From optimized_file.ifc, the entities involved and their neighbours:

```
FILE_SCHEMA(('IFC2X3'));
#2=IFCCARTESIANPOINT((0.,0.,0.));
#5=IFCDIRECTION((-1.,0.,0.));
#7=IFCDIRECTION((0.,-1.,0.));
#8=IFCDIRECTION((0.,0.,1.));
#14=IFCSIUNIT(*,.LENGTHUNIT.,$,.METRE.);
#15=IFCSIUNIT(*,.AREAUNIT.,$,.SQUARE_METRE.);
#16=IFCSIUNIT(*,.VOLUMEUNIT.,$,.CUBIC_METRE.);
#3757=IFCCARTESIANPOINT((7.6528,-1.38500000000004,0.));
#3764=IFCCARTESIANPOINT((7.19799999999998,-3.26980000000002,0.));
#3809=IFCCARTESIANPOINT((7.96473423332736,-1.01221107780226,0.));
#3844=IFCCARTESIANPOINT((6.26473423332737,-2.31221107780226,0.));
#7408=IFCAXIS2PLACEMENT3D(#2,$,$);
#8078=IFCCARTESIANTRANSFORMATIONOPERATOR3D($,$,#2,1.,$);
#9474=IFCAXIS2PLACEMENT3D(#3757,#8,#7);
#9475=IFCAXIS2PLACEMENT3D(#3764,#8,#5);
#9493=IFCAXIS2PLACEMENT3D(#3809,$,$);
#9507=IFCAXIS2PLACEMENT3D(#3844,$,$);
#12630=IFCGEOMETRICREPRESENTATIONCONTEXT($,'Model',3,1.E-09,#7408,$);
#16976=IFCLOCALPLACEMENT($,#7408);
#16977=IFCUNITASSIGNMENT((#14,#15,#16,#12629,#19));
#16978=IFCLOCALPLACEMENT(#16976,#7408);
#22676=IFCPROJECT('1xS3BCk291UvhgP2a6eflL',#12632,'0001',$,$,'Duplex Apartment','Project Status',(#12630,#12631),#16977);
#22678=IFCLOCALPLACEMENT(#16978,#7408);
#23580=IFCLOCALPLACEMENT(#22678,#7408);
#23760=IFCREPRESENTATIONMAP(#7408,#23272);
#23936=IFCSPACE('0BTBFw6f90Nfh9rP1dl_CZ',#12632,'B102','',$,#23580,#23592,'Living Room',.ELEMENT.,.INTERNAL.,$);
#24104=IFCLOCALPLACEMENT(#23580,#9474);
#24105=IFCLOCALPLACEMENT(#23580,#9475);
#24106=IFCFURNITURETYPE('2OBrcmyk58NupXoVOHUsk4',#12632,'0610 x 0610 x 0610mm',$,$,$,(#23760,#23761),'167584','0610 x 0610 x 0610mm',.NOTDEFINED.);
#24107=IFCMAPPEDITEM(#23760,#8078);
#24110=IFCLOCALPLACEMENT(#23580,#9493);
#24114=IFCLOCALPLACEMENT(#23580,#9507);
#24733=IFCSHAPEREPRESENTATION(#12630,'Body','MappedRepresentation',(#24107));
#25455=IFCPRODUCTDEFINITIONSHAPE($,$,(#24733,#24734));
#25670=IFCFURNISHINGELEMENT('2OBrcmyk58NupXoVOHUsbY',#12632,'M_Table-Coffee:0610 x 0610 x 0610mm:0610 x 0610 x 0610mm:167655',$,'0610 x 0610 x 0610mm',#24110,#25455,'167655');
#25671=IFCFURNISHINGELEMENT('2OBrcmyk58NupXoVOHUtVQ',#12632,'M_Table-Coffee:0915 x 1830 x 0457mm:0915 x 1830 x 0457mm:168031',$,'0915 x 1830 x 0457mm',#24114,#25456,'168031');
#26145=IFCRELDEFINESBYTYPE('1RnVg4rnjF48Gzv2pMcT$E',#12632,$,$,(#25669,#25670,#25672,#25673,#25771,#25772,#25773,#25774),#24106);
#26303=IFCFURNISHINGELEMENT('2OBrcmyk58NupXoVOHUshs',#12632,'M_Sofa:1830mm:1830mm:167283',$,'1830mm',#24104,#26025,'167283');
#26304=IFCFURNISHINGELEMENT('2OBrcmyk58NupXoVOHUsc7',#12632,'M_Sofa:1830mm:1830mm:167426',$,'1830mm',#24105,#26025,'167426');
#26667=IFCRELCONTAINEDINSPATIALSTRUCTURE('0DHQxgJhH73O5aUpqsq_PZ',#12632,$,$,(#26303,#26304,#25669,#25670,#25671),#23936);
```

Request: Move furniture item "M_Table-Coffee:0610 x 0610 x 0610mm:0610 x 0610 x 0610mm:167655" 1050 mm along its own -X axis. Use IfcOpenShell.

```python
import ifcopenshell
import ifcopenshell.api.geometry
import ifcopenshell.util.placement
import ifcopenshell.util.unit

model = ifcopenshell.open("optimized_file.ifc")
unit_scale = ifcopenshell.util.unit.calculate_unit_scale(model)

item = model.by_guid("2OBrcmyk58NupXoVOHUsbY")
matrix = ifcopenshell.util.placement.get_local_placement(item.ObjectPlacement)
matrix[:3, 3] -= matrix[:3, 0] * 1.05 / unit_scale
ifcopenshell.api.geometry.edit_object_placement(model, product=item, matrix=matrix, is_si=False)

print(ifcopenshell.util.placement.get_local_placement(item.ObjectPlacement).round(3) + 0.0)

model.write("optimized_file_v2.ifc")
```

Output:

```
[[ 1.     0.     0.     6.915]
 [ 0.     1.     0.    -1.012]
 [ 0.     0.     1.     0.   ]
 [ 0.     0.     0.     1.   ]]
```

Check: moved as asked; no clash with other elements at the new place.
